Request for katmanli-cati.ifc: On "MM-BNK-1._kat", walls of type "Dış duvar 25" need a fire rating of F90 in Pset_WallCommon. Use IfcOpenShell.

First a look at what the model holds.

```python
import ifcopenshell
import ifcopenshell.util.element

model = ifcopenshell.open("katmanli-cati.ifc")
print(model.schema)
storey = next(s for s in model.by_type("IfcBuildingStorey") if s.Name == "MM-BNK-1._kat")
walls = [e for e in ifcopenshell.util.element.get_decomposition(storey) if e.is_a("IfcWall")]
seen = {}
for e in walls:
    element_type = ifcopenshell.util.element.get_type(e)
    key = (element_type.Name if element_type != e and element_type else None, ifcopenshell.util.element.get_pset(e, "Pset_WallCommon", "FireRating"))
    seen[key] = seen.get(key, 0) + 1
for (name, value), count in sorted(seen.items(), key=str):
    print(count, "x", name, "|", value)
```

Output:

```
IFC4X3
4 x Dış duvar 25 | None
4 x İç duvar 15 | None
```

```python
import ifcopenshell
import ifcopenshell.api.pset
import ifcopenshell.util.element

model = ifcopenshell.open("katmanli-cati.ifc")

storey = next(s for s in model.by_type("IfcBuildingStorey") if s.Name == "MM-BNK-1._kat")
walls = [e for e in ifcopenshell.util.element.get_decomposition(storey) if e.is_a("IfcWall")]

count = 0
for e in walls:
    element_type = ifcopenshell.util.element.get_type(e)
    if element_type in (None, e) or element_type.Name != "Dış duvar 25":
        continue
    # add_pset returns the element's existing set when there is one.
    pset = ifcopenshell.api.pset.add_pset(model, product=e, name="Pset_WallCommon")
    ifcopenshell.api.pset.edit_pset(model, pset=pset, properties={"FireRating": "F90"})
    count += 1

print(count, "walls updated")

model.write("katmanli-cati_edited.ifc")
```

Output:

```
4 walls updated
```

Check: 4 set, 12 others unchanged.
